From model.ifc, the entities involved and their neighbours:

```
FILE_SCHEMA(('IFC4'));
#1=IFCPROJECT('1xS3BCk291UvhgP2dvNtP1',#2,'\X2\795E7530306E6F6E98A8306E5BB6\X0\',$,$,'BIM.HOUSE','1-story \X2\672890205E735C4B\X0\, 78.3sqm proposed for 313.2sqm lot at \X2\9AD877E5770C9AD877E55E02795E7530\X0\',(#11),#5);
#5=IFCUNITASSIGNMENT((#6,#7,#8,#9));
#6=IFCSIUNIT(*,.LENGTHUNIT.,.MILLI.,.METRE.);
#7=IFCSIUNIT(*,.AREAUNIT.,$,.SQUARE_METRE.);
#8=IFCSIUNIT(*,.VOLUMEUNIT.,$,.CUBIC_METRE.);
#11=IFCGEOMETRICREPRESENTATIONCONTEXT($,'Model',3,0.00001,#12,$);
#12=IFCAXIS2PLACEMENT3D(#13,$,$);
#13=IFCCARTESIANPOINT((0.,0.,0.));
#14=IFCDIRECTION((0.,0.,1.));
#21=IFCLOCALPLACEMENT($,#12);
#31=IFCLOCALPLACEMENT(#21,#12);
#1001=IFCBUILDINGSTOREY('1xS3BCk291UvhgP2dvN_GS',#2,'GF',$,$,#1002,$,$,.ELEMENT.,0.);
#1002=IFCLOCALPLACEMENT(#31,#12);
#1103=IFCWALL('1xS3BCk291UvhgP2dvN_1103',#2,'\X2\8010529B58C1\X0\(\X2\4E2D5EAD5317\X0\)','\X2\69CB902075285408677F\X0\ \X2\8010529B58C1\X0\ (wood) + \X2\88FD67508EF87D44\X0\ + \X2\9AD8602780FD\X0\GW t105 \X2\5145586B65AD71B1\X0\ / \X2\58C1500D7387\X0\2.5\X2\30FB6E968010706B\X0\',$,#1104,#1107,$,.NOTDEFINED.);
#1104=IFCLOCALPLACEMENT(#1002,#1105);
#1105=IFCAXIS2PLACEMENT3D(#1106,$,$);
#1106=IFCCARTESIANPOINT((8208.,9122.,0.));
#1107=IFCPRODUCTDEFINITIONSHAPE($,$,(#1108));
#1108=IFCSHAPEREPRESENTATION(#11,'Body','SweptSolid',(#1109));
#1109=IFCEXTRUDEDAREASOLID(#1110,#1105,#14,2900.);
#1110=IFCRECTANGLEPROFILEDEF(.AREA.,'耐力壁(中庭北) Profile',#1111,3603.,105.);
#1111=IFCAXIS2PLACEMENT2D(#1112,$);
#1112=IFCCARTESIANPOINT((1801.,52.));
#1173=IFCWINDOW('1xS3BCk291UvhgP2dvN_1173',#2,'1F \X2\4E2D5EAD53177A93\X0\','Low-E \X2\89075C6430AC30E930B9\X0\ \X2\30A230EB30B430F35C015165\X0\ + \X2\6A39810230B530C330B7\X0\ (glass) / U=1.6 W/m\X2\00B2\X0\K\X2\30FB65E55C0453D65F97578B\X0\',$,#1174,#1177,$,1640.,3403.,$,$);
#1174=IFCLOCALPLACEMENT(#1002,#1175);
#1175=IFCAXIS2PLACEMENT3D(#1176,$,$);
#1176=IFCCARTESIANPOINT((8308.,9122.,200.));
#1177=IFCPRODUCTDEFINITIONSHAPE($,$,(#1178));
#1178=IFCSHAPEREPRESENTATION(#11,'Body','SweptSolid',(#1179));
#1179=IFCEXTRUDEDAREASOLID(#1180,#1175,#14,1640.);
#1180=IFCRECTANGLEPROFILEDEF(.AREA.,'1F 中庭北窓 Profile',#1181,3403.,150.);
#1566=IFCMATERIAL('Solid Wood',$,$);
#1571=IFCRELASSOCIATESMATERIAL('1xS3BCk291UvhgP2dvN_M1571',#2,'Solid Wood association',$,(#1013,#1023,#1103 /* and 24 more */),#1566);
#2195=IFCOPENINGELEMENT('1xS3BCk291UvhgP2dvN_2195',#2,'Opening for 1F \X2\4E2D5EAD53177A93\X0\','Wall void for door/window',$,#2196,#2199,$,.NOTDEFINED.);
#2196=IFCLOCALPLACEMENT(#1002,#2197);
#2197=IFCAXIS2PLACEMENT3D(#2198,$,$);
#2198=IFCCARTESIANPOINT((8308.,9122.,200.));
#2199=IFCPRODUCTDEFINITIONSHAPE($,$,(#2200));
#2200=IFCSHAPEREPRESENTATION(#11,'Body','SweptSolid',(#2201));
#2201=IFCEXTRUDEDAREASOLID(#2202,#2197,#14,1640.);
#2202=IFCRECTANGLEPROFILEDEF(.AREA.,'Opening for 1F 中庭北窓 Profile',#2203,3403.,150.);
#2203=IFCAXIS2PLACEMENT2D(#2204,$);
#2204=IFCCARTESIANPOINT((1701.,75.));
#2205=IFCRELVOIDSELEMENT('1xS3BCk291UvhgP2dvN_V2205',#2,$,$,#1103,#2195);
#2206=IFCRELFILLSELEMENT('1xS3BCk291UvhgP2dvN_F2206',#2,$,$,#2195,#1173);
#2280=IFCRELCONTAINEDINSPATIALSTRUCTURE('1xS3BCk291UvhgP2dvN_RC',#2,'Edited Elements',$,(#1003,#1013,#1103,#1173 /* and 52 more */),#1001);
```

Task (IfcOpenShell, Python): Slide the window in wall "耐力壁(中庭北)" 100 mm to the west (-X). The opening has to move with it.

```python
import ifcopenshell
import ifcopenshell.api.geometry
import ifcopenshell.util.placement

model = ifcopenshell.open("model.ifc")

window = model.by_guid("1xS3BCk291UvhgP2dvN_1173")
opening = window.FillsVoids[0].RelatingOpeningElement
wall = opening.VoidsElements[0].RelatingBuildingElement

wall_matrix = ifcopenshell.util.placement.get_local_placement(wall.ObjectPlacement)
shift = wall_matrix[:3, 0] * -100.0
before = ifcopenshell.util.placement.get_local_placement(window.ObjectPlacement)[:3, 3].copy()

# The window is not placed relative to its opening, so move both.
for product in (opening, window):
    matrix = ifcopenshell.util.placement.get_local_placement(product.ObjectPlacement)
    matrix[:3, 3] += shift
    ifcopenshell.api.geometry.edit_object_placement(model, product=product, matrix=matrix, is_si=False)

after = ifcopenshell.util.placement.get_local_placement(window.ObjectPlacement)[:3, 3]
print("window moved by", (after - before).round(3) + 0.0)

model.write("model_rev.ifc")
```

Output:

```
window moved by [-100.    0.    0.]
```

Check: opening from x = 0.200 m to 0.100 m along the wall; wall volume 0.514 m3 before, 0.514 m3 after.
